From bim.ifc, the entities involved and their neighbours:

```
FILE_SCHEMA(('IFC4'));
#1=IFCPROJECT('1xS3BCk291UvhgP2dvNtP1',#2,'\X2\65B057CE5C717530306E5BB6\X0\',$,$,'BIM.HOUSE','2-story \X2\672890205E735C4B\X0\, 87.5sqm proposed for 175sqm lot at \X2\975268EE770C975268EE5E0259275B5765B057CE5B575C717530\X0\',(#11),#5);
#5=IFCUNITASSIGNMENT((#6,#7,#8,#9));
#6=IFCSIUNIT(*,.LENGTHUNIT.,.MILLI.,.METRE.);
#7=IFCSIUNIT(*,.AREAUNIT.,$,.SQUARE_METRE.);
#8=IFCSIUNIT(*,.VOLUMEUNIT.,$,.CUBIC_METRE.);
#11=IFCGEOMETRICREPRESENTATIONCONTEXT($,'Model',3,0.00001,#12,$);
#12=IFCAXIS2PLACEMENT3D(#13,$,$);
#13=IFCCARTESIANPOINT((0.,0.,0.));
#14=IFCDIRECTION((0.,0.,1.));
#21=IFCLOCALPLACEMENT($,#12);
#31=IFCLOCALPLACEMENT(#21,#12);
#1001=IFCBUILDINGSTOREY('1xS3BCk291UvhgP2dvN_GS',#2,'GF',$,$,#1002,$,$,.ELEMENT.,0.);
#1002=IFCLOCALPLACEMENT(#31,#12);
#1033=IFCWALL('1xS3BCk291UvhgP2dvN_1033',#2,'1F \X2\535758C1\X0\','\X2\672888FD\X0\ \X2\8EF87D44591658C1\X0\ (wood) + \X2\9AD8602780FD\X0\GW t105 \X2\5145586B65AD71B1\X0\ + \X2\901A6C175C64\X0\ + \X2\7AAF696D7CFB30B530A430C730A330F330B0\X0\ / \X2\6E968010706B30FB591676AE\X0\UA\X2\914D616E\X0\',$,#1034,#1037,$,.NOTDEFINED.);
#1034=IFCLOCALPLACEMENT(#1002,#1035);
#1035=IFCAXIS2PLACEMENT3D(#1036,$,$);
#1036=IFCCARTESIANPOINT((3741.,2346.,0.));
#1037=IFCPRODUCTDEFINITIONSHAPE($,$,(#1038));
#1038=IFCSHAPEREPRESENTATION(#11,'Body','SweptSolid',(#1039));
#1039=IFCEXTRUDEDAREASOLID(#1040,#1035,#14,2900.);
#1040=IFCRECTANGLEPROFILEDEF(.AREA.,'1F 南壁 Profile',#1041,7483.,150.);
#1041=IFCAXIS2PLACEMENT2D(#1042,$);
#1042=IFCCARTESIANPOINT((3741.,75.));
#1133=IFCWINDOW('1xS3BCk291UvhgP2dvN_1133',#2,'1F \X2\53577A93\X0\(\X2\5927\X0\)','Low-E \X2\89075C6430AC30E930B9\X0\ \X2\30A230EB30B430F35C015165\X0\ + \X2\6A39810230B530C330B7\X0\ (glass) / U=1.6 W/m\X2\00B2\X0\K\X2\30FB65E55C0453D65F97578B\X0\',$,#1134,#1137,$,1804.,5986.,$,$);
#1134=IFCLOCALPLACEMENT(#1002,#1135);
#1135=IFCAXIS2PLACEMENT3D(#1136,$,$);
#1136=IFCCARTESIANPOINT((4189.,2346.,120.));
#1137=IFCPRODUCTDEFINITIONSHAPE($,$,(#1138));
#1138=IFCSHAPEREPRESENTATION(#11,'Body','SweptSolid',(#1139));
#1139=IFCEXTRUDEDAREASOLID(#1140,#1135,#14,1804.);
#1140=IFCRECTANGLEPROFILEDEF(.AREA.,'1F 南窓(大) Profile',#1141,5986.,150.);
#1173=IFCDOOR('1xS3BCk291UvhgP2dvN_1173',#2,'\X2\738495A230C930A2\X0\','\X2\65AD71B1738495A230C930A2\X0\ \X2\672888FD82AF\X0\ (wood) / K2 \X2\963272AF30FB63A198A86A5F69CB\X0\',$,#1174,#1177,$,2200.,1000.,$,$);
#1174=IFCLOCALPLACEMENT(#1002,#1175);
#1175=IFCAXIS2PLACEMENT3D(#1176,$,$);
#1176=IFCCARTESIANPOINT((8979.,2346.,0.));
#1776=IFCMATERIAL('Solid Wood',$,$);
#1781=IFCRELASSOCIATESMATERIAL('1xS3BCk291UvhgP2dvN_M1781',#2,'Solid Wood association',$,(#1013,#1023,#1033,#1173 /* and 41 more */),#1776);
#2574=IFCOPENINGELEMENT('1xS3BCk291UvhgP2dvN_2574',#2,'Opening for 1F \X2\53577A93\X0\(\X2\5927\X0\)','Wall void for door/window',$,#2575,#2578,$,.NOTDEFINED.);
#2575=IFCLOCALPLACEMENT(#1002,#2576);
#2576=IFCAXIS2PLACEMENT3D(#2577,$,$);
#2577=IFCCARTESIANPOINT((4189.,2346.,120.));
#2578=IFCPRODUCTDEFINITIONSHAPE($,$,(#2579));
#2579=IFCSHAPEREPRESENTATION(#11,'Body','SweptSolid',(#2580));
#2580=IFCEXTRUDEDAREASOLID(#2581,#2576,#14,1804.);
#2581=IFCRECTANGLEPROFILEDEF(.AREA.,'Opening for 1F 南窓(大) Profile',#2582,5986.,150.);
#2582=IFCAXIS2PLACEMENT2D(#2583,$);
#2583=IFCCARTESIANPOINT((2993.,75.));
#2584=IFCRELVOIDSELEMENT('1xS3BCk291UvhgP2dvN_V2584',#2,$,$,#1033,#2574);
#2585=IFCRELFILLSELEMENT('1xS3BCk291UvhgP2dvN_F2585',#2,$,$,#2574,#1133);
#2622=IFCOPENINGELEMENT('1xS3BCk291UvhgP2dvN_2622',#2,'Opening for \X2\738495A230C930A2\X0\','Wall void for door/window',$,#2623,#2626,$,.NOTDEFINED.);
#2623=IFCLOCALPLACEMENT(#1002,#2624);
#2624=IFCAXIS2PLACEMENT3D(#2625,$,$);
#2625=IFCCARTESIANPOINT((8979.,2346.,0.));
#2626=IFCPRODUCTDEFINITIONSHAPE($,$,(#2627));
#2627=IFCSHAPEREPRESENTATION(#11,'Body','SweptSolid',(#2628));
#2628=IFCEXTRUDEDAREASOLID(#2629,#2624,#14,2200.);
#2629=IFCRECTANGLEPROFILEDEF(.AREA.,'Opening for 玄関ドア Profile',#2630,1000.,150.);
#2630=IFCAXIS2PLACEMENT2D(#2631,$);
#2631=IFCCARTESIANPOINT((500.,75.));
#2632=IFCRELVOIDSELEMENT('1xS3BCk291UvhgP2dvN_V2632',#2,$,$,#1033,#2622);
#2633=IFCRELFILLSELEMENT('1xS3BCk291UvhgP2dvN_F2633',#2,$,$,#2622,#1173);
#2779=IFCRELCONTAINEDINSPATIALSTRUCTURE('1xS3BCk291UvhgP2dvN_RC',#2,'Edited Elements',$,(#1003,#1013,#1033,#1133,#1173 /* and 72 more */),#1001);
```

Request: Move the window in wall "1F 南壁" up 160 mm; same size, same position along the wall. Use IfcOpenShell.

```python
import numpy as np
import ifcopenshell
import ifcopenshell.api.geometry
import ifcopenshell.util.placement
import ifcopenshell.util.unit

model = ifcopenshell.open("bim.ifc")
unit_scale = ifcopenshell.util.unit.calculate_unit_scale(model)

window = model.by_guid("1xS3BCk291UvhgP2dvN_1133")
opening = window.FillsVoids[0].RelatingOpeningElement
dz = 160.0

shift = np.array([0.0, 0.0, dz])
# The window is not placed relative to its opening, so move both.
for product in (opening, window):
    matrix = ifcopenshell.util.placement.get_local_placement(product.ObjectPlacement)
    matrix[:3, 3] += shift
    ifcopenshell.api.geometry.edit_object_placement(model, product=product, matrix=matrix, is_si=False)

print(f"moved by {dz * unit_scale:+.3f} m")

model.write("bim_edited.ifc")
```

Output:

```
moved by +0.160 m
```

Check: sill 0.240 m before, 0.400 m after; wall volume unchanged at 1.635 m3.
